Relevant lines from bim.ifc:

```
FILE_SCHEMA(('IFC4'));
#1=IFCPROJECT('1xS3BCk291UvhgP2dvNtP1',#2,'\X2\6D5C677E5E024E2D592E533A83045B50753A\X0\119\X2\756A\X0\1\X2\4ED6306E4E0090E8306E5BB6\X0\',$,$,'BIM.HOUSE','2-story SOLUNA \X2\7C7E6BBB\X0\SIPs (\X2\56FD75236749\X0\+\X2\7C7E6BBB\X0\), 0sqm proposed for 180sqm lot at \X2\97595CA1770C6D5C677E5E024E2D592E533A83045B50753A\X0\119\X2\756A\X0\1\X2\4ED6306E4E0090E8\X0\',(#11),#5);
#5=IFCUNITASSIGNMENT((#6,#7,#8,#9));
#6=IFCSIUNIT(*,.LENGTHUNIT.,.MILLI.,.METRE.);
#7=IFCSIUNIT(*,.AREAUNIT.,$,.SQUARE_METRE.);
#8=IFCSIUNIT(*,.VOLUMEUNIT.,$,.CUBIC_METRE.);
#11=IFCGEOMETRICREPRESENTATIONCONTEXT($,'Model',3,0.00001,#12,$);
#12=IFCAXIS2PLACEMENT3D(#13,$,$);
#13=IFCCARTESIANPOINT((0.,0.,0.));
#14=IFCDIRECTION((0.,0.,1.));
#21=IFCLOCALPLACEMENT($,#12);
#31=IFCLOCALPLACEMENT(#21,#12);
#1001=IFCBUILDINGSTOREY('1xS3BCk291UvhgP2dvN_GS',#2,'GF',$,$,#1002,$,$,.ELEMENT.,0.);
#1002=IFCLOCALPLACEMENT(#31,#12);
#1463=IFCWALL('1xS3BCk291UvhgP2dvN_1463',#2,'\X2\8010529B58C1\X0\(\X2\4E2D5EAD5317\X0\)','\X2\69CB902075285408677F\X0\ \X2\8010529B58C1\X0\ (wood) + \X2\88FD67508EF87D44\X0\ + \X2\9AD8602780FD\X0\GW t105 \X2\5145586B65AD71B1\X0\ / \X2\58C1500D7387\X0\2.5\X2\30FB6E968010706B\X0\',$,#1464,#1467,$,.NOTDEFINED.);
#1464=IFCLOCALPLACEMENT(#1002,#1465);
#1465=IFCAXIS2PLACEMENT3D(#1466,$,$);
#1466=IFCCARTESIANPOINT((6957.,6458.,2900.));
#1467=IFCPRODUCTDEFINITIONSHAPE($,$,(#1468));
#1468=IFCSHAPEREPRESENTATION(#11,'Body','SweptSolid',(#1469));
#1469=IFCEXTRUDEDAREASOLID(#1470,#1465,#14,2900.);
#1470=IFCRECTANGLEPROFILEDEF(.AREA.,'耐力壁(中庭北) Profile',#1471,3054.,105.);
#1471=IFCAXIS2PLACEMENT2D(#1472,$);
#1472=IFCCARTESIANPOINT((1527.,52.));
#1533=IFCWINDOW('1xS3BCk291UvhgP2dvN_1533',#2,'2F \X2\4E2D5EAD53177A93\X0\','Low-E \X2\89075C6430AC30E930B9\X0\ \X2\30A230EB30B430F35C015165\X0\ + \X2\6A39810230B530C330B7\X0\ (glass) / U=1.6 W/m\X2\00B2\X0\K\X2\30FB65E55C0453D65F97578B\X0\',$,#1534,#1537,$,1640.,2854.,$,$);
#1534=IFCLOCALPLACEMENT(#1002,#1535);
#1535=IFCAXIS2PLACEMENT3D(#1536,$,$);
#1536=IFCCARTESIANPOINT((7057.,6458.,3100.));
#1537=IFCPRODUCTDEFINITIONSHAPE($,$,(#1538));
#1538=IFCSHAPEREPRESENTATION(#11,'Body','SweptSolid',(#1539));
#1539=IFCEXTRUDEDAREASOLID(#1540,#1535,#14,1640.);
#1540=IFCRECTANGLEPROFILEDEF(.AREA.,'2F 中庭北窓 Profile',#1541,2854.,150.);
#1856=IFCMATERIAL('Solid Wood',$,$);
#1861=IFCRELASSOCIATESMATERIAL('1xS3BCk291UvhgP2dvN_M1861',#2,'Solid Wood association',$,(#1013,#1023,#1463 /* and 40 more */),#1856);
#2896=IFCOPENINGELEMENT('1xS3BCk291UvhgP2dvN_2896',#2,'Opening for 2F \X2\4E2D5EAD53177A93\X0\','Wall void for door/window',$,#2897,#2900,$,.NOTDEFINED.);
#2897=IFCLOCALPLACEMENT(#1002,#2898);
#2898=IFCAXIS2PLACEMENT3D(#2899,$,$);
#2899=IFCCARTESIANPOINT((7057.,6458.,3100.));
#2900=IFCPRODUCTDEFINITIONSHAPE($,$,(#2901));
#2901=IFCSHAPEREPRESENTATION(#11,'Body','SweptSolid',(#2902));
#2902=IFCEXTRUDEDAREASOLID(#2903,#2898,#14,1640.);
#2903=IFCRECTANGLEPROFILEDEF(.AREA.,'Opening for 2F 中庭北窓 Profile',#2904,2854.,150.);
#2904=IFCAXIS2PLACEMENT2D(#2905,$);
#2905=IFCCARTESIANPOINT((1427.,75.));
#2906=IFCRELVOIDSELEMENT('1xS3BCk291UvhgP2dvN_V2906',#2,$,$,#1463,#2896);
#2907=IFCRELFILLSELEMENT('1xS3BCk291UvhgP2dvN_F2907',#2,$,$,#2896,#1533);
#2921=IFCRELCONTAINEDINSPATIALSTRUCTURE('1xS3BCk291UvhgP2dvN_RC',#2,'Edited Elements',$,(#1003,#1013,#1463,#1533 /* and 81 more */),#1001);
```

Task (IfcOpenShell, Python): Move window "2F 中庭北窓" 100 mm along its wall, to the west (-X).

```python
import ifcopenshell
import ifcopenshell.api.geometry
import ifcopenshell.util.placement
import ifcopenshell.util.unit

model = ifcopenshell.open("bim.ifc")
unit_scale = ifcopenshell.util.unit.calculate_unit_scale(model)

window = model.by_guid("1xS3BCk291UvhgP2dvN_1533")
opening = window.FillsVoids[0].RelatingOpeningElement
wall = opening.VoidsElements[0].RelatingBuildingElement

wall_matrix = ifcopenshell.util.placement.get_local_placement(wall.ObjectPlacement)
shift = wall_matrix[:3, 0] * -0.1 / unit_scale
before = ifcopenshell.util.placement.get_local_placement(window.ObjectPlacement)[:3, 3].copy()

# The window is not placed relative to its opening, so move both.
for product in (opening, window):
    matrix = ifcopenshell.util.placement.get_local_placement(product.ObjectPlacement)
    matrix[:3, 3] += shift
    ifcopenshell.api.geometry.edit_object_placement(model, product=product, matrix=matrix, is_si=False)

after = ifcopenshell.util.placement.get_local_placement(window.ObjectPlacement)[:3, 3]
print("window moved by", (after - before).round(3) + 0.0)

model.write("bim_v2.ifc")
```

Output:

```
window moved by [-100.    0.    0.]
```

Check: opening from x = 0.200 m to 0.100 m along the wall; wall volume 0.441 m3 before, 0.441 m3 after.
